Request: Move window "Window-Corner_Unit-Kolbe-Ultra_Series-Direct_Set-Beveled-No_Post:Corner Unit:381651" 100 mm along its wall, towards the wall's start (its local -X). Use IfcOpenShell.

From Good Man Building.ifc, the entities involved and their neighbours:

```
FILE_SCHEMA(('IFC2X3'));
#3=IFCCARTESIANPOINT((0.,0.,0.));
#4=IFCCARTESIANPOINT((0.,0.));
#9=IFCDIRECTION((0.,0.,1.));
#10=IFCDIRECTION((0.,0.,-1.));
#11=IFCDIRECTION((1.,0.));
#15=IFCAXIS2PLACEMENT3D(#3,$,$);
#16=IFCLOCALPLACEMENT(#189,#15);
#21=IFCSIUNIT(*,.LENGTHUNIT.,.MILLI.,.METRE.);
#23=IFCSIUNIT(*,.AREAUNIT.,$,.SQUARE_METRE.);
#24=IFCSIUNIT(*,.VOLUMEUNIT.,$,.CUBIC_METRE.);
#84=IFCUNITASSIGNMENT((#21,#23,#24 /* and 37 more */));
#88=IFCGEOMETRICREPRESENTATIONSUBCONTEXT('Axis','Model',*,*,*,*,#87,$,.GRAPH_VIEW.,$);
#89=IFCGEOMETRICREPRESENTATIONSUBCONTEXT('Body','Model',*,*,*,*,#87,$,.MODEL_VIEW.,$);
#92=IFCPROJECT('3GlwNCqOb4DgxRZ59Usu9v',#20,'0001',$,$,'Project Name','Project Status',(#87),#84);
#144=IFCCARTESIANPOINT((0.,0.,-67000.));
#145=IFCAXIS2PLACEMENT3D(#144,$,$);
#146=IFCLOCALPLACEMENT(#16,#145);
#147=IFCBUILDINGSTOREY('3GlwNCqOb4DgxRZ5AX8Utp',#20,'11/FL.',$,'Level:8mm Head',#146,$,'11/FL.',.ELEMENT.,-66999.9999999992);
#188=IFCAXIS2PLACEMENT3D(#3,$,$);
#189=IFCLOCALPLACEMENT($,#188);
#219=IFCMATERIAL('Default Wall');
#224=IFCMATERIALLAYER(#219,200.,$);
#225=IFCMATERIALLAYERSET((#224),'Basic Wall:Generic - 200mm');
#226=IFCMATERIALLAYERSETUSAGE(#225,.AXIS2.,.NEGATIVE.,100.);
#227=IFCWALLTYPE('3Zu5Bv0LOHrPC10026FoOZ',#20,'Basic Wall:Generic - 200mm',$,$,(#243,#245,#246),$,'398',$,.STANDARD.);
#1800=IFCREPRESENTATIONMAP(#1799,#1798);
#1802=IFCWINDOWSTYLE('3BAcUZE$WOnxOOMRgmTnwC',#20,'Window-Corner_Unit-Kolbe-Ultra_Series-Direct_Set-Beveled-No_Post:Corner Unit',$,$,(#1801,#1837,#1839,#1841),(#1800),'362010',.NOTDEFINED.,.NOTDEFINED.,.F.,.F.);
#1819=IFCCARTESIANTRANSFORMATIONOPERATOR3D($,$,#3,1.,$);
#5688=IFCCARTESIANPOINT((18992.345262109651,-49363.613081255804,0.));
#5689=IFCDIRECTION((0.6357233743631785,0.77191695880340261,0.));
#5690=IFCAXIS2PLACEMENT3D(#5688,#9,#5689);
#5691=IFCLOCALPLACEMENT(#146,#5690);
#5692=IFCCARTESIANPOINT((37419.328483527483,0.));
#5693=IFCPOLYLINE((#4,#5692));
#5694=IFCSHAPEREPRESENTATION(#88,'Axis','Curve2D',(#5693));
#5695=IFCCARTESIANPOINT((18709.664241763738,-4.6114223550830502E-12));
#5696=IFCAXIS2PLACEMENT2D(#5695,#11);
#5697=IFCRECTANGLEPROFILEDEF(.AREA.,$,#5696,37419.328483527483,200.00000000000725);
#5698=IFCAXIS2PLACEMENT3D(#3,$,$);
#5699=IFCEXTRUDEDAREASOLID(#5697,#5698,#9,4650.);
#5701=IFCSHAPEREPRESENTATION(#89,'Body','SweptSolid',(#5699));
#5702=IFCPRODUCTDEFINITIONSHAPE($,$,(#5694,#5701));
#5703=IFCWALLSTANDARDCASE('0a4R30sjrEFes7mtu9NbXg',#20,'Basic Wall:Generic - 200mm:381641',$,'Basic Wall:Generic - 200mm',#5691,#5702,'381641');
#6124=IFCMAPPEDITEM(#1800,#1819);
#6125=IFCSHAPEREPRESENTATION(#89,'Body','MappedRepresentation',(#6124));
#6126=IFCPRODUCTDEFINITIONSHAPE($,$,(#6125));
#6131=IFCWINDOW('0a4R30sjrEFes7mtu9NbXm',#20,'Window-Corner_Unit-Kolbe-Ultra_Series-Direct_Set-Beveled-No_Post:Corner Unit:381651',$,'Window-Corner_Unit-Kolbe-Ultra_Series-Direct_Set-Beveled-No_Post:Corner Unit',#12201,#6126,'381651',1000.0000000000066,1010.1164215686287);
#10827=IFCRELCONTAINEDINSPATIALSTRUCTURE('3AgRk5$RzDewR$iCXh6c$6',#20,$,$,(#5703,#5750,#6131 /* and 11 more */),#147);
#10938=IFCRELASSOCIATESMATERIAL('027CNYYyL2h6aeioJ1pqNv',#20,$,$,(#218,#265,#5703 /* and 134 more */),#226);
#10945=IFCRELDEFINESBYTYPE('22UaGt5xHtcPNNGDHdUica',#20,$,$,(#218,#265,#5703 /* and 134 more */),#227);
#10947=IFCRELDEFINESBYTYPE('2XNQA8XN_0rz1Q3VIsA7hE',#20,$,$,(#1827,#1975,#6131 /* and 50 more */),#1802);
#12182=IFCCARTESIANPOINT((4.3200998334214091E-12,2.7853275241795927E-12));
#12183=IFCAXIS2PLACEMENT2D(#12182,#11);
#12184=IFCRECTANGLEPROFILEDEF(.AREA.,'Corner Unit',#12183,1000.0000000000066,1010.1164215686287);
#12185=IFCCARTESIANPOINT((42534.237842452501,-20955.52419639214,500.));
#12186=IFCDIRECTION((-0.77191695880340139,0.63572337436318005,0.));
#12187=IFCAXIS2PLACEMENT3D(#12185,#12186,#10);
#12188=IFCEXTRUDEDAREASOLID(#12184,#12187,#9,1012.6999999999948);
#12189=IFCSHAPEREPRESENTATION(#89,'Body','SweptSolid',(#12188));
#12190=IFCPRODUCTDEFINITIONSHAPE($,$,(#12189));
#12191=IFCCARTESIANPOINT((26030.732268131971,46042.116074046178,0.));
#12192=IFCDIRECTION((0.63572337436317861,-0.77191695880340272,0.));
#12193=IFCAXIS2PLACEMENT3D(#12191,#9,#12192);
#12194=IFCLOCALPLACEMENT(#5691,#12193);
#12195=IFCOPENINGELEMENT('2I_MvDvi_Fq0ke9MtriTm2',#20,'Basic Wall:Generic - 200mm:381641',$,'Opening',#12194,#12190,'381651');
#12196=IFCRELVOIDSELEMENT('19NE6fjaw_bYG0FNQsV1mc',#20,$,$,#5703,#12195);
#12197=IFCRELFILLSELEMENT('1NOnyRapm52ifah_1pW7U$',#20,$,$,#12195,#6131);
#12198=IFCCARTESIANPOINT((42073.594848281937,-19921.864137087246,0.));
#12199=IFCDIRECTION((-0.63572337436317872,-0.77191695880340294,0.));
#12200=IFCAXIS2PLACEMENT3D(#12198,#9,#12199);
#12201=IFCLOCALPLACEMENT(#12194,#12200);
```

```python
import ifcopenshell
import ifcopenshell.api.geometry
import ifcopenshell.util.placement
import ifcopenshell.util.unit

model = ifcopenshell.open("Good Man Building.ifc")
unit_scale = ifcopenshell.util.unit.calculate_unit_scale(model)

window = model.by_id(6131)
opening = window.FillsVoids[0].RelatingOpeningElement
wall = opening.VoidsElements[0].RelatingBuildingElement

wall_matrix = ifcopenshell.util.placement.get_local_placement(wall.ObjectPlacement)
shift = wall_matrix[:3, 0] * -0.1 / unit_scale
before = ifcopenshell.util.placement.get_local_placement(window.ObjectPlacement)[:3, 3].copy()

# The window is placed relative to its opening, so it follows when the opening moves.
matrix = ifcopenshell.util.placement.get_local_placement(opening.ObjectPlacement)
matrix[:3, 3] += shift
ifcopenshell.api.geometry.edit_object_placement(
    model, product=opening, matrix=matrix, is_si=False, should_transform_children=True
)

after = ifcopenshell.util.placement.get_local_placement(window.ObjectPlacement)[:3, 3]
print("window moved by", (after - before).round(3) + 0.0)

model.write("Good Man Building_edited.ifc")
```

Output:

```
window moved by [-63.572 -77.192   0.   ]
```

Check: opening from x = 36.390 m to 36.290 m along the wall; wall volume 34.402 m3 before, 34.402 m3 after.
